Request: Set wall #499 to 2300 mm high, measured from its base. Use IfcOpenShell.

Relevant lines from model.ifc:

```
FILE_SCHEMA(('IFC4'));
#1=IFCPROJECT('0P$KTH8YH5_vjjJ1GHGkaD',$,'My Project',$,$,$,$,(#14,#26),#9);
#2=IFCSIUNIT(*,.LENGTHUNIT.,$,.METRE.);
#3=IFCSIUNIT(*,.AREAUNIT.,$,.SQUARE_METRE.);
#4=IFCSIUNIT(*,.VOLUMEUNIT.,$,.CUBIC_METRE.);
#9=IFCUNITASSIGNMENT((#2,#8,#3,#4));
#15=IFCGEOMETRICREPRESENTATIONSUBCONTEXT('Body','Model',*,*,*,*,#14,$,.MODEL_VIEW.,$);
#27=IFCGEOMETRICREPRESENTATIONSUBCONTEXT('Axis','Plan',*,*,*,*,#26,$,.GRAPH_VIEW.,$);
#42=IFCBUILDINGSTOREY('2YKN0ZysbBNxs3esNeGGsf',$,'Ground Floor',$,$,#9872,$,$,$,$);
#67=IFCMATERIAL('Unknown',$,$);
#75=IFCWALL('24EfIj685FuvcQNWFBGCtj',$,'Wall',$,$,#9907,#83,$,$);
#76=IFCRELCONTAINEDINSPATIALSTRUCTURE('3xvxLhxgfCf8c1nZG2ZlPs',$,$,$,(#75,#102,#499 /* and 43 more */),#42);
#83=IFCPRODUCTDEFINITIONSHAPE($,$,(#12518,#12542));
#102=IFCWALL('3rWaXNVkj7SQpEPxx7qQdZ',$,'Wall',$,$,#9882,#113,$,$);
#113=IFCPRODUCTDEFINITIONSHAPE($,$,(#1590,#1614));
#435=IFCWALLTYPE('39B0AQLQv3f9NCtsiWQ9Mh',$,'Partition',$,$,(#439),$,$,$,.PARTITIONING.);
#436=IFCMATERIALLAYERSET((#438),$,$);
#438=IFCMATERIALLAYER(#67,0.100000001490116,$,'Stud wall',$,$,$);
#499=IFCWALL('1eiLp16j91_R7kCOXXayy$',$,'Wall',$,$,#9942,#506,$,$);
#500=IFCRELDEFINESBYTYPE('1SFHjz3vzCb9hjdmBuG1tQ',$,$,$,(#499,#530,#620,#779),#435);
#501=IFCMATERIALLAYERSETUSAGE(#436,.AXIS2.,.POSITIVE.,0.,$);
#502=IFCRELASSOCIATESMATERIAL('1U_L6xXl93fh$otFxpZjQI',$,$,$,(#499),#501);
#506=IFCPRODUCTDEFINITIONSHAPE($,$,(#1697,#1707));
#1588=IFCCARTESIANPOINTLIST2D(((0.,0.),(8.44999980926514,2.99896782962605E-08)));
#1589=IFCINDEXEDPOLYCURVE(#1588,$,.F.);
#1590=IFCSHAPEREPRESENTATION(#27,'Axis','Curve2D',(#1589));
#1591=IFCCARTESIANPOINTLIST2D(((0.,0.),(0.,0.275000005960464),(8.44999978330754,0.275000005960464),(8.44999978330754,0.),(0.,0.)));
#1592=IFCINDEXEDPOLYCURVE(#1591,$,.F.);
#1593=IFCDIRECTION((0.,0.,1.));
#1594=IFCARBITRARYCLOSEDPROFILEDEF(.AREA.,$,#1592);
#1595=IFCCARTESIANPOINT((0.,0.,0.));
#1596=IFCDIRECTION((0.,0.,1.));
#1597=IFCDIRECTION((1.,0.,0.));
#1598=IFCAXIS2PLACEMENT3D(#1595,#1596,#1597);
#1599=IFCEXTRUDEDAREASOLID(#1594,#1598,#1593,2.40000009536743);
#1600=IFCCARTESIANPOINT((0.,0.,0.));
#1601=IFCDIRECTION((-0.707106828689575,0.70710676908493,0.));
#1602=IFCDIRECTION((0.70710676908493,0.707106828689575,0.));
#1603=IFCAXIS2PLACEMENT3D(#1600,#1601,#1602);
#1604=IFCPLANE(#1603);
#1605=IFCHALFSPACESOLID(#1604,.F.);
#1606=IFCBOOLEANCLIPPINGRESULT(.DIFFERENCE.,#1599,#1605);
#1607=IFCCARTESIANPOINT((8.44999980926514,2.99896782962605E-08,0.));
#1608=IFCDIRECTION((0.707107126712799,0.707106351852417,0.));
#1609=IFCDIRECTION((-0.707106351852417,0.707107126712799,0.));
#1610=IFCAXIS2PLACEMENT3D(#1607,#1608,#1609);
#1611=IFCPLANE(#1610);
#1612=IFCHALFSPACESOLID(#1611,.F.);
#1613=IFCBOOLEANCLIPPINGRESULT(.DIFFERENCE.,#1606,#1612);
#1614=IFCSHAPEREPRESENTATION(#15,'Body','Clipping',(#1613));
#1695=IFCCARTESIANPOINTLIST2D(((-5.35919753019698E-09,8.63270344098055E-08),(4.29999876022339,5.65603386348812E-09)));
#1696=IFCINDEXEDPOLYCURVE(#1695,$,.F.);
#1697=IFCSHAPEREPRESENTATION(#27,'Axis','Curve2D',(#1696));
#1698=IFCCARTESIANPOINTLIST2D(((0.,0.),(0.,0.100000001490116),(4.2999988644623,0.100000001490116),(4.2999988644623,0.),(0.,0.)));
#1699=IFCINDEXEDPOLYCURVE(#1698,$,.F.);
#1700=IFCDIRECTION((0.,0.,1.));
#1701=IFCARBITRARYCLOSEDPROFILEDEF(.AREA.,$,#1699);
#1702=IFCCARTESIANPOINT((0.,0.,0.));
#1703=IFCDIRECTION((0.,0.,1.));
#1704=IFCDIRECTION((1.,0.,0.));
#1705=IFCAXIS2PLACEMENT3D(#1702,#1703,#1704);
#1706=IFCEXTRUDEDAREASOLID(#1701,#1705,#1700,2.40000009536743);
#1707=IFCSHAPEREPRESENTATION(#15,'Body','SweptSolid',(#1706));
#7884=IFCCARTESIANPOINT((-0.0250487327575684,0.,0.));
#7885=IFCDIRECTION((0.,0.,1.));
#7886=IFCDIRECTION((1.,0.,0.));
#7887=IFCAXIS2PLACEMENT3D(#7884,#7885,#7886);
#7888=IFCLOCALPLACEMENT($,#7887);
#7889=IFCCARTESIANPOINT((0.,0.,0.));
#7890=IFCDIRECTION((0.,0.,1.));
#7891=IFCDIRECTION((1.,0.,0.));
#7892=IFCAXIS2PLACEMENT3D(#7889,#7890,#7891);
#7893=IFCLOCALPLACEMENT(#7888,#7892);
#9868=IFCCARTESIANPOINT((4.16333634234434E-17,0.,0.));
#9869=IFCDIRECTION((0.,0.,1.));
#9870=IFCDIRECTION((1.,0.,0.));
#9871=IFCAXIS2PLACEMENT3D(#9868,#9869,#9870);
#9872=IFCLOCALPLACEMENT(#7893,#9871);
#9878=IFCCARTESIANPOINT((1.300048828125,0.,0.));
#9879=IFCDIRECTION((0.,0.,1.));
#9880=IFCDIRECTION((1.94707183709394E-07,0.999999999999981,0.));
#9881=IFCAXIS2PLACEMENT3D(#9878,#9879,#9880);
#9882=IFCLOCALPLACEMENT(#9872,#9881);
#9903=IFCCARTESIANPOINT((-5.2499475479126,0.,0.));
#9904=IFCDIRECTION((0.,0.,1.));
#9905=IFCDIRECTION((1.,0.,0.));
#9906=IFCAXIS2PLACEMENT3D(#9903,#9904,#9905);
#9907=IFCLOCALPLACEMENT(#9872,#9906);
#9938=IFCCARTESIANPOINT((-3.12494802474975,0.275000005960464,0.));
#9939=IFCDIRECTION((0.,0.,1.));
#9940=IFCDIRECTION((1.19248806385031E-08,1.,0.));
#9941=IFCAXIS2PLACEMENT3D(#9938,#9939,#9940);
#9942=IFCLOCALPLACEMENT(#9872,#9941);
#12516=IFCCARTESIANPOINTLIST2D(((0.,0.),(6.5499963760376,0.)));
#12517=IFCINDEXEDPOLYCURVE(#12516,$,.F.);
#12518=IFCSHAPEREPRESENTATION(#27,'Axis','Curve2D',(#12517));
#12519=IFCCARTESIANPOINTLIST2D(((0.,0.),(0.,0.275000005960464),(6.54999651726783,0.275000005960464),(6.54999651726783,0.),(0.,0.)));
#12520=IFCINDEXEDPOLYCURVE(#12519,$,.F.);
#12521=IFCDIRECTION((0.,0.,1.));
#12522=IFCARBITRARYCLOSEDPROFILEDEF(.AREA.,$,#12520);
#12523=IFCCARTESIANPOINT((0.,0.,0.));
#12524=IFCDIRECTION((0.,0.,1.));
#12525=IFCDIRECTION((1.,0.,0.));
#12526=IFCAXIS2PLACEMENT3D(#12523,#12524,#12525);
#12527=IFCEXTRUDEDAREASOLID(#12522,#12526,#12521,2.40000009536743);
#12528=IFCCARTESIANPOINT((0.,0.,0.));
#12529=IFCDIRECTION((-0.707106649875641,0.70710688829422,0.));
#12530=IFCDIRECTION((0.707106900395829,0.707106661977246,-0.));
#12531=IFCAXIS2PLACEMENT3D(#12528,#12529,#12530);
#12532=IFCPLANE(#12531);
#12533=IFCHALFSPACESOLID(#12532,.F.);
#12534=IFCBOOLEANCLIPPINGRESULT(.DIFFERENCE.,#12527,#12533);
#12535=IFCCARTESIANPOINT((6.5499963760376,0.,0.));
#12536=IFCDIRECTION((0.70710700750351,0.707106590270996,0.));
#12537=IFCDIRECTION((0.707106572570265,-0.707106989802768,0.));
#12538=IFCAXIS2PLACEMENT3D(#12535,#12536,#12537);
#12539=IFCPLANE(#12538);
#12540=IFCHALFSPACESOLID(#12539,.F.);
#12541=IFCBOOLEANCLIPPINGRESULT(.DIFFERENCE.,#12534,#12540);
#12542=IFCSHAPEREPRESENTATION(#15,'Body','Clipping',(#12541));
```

```python
import ifcopenshell
import ifcopenshell.geom
import ifcopenshell.util.representation
import ifcopenshell.util.shape

model = ifcopenshell.open("model.ifc")
settings = ifcopenshell.geom.settings()


def volume(element):
    """Net volume in cubic metres, openings subtracted."""
    shape = ifcopenshell.geom.create_shape(settings, element)
    return ifcopenshell.util.shape.get_volume(shape.geometry)


wall = model.by_guid("1eiLp16j91_R7kCOXXayy$")
before = volume(wall)

body = ifcopenshell.util.representation.get_representation(wall, "Model", "Body")
solid = body.Items[0]
old_height = solid.Depth
solid.Depth = 2.3
after = volume(wall)

print(f"height {old_height:g} -> {solid.Depth:g}, volume {before:.3f} -> {after:.3f} m3")

model.write("model_v2.ifc")
```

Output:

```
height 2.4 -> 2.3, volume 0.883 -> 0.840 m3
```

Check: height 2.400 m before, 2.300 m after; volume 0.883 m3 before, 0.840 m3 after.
